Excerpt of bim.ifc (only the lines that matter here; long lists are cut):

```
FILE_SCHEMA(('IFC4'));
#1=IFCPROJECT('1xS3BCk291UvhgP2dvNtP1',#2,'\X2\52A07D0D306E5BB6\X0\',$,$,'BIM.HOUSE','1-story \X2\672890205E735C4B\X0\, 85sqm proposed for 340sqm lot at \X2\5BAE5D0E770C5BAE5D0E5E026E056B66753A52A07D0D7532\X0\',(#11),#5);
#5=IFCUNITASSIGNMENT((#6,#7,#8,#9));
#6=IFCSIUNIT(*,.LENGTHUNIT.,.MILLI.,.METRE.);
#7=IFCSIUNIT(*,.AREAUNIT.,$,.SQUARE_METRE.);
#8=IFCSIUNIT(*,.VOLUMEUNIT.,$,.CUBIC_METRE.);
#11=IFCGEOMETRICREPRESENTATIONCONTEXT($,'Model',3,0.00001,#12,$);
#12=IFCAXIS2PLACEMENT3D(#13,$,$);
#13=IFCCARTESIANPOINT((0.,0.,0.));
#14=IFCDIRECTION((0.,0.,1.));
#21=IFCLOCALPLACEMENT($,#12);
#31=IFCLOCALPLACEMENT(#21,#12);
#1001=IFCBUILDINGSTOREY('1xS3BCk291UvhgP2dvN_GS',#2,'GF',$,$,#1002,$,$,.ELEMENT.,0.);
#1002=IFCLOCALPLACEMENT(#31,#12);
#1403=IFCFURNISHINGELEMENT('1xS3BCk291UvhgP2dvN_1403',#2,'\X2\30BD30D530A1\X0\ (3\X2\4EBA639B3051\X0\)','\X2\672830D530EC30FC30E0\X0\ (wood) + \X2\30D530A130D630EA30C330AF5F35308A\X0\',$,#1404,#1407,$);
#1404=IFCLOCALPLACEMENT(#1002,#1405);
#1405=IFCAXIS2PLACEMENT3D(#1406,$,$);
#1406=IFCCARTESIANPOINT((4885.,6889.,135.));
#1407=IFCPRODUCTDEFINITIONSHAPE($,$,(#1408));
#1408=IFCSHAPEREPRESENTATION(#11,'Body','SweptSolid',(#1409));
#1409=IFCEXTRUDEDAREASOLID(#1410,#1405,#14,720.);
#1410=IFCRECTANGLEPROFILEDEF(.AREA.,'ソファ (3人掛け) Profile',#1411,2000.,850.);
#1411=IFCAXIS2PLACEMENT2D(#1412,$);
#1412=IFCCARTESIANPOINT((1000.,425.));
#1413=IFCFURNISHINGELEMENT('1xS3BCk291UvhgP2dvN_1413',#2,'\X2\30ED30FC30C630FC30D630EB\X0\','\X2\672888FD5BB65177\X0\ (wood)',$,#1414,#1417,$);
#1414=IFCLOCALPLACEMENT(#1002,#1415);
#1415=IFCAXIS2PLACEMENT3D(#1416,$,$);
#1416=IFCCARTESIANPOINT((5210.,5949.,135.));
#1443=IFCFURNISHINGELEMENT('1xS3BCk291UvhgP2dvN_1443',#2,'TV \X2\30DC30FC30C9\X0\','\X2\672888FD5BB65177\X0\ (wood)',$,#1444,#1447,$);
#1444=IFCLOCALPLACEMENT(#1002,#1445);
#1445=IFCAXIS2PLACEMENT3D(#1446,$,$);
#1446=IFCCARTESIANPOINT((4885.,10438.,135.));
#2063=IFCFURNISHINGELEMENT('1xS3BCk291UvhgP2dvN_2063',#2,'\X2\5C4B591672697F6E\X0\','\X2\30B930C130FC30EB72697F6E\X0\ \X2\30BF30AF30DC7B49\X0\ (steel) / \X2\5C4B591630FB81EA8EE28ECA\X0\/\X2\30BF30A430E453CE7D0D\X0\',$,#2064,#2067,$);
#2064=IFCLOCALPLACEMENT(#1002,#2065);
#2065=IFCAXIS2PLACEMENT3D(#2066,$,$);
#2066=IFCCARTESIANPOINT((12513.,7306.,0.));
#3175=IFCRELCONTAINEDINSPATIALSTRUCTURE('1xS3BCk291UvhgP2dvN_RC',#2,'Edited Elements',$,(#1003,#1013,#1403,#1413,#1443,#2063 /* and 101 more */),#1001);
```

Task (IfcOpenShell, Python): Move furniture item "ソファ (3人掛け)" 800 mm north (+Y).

```python
import ifcopenshell
import ifcopenshell.api.geometry
import ifcopenshell.util.placement
import ifcopenshell.util.unit

model = ifcopenshell.open("bim.ifc")
unit_scale = ifcopenshell.util.unit.calculate_unit_scale(model)

item = model.by_id(1403)
matrix = ifcopenshell.util.placement.get_local_placement(item.ObjectPlacement)
matrix[1, 3] += 0.8 / unit_scale
ifcopenshell.api.geometry.edit_object_placement(model, product=item, matrix=matrix, is_si=False)

print(ifcopenshell.util.placement.get_local_placement(item.ObjectPlacement).round(3) + 0.0)

model.write("bim_rev.ifc")
```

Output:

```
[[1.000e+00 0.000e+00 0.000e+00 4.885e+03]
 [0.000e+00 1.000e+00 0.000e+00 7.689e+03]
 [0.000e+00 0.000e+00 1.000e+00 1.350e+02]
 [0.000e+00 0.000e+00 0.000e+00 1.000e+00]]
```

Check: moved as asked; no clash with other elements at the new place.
